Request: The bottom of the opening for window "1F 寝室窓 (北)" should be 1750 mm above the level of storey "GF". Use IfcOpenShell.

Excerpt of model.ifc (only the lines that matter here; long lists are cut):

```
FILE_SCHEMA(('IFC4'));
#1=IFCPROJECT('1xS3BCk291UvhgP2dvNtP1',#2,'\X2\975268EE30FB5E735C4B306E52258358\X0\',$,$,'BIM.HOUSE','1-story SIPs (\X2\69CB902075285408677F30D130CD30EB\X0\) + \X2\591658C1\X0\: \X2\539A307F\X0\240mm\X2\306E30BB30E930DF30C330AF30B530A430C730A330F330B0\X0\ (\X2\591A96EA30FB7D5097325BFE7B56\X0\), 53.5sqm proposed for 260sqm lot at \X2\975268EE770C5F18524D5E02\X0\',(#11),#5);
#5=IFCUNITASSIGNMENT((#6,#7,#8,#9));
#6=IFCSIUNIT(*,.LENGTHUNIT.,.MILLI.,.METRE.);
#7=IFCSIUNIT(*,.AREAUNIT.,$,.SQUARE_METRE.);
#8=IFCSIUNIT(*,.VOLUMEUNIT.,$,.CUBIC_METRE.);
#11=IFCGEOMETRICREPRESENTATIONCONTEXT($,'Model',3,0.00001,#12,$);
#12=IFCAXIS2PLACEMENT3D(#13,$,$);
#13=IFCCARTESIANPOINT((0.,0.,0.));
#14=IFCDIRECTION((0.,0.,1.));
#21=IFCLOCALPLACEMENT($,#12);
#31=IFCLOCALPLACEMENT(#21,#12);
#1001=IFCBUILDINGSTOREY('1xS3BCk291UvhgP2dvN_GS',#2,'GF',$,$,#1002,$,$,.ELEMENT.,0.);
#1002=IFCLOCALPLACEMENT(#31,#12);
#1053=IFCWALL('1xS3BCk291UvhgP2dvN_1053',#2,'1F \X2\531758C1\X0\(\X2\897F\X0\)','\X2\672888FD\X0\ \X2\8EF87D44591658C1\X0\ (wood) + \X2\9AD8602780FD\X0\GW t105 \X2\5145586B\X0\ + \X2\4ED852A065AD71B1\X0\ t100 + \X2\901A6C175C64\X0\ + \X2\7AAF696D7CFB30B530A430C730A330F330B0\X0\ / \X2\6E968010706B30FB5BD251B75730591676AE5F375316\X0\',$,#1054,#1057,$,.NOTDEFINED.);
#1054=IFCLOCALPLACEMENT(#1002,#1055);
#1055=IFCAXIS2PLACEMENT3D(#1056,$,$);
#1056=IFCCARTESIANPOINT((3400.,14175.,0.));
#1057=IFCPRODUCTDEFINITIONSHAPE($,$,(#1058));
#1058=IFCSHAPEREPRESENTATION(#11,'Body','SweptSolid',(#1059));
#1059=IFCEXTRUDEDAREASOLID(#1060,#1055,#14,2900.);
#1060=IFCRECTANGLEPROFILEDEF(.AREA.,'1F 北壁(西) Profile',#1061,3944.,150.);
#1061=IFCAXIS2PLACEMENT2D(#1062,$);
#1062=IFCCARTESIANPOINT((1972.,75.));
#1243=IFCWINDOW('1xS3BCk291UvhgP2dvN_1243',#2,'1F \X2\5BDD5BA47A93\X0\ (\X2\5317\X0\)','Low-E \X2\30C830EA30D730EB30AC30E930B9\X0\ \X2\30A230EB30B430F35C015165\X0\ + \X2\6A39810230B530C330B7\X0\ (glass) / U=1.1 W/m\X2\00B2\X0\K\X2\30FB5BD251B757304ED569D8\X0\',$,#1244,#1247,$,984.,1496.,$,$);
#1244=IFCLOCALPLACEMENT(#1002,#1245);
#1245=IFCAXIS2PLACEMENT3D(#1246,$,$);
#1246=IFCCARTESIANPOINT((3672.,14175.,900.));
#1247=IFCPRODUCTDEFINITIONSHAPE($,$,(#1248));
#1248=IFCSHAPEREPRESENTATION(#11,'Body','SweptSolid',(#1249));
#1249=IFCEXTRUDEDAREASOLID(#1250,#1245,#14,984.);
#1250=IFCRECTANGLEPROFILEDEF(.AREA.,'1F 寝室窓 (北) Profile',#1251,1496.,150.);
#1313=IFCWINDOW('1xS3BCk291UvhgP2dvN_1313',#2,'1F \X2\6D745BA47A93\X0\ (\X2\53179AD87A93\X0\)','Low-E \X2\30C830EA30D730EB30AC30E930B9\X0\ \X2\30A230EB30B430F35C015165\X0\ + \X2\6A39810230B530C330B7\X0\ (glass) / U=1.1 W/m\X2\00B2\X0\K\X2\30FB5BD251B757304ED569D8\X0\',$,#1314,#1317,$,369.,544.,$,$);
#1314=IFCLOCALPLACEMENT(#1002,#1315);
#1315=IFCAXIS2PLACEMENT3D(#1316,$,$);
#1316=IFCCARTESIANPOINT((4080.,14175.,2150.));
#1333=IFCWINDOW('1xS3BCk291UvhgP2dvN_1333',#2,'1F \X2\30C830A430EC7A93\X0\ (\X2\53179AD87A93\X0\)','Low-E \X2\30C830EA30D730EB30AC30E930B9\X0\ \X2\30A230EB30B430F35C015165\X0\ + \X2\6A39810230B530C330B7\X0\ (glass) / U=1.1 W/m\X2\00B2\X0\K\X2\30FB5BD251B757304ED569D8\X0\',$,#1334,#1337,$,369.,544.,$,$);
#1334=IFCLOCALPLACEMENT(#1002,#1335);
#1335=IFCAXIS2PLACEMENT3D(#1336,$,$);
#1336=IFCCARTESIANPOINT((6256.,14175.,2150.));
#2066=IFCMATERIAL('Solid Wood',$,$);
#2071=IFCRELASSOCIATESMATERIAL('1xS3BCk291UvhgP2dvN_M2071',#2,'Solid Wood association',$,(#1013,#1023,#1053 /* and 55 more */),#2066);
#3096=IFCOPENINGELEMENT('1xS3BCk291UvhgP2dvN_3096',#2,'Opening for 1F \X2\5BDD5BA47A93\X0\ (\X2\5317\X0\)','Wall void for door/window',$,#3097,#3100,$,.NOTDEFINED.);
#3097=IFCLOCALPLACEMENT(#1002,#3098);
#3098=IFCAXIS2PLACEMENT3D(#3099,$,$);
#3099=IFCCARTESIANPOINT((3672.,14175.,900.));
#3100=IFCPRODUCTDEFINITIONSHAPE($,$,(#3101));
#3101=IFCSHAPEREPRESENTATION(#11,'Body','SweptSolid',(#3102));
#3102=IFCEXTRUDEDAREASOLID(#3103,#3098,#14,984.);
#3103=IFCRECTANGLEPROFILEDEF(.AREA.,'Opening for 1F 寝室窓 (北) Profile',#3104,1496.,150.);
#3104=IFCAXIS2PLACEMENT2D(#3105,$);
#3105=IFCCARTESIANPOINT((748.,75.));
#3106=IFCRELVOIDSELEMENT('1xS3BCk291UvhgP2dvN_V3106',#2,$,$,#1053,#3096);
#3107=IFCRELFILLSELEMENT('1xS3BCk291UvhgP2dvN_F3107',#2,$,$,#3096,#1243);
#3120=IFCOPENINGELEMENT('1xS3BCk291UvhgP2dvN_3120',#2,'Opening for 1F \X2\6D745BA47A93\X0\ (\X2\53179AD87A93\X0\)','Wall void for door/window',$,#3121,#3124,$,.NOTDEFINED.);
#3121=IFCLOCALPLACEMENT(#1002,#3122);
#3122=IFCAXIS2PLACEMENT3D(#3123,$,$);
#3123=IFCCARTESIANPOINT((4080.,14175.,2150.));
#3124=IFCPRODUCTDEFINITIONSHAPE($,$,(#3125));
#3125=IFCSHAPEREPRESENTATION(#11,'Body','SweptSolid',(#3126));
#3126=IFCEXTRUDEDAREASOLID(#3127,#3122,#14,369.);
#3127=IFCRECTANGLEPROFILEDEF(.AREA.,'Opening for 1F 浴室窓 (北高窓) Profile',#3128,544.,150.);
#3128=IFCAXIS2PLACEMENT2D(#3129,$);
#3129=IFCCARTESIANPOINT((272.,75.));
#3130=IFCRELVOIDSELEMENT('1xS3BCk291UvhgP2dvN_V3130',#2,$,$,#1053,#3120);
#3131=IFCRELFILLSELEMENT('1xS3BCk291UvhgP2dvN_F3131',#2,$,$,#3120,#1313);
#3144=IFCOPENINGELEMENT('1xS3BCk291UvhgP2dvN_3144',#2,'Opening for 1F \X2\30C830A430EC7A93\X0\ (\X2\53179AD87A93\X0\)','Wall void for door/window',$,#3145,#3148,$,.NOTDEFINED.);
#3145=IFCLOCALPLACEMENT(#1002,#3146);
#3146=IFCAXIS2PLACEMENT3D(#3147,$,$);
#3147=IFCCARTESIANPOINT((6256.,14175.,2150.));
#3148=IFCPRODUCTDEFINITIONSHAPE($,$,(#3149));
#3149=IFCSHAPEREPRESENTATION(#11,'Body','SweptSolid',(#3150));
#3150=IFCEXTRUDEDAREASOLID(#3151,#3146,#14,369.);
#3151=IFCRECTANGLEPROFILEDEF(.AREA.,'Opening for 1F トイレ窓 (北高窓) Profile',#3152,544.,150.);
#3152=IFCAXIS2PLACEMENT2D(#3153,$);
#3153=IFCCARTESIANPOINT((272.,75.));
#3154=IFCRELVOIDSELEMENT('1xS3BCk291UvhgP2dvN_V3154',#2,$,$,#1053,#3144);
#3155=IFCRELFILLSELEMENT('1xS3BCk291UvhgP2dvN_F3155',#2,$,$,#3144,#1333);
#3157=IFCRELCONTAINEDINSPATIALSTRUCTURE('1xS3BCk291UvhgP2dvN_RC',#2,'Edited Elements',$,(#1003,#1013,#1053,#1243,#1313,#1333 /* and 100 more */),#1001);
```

```python
import numpy as np
import ifcopenshell
import ifcopenshell.api.geometry
import ifcopenshell.geom
import ifcopenshell.util.element
import ifcopenshell.util.placement
import ifcopenshell.util.shape
import ifcopenshell.util.unit

model = ifcopenshell.open("model.ifc")
unit_scale = ifcopenshell.util.unit.calculate_unit_scale(model)

window = model.by_guid("1xS3BCk291UvhgP2dvN_1243")
opening = window.FillsVoids[0].RelatingOpeningElement
storey = ifcopenshell.util.element.get_container(window, ifc_class="IfcBuildingStorey")
level = ifcopenshell.util.placement.get_local_placement(storey.ObjectPlacement)[2, 3]

# The opening's origin need not be at the sill, so measure its lowest point.
shape = ifcopenshell.geom.create_shape(ifcopenshell.geom.settings(), opening)
bottom = ifcopenshell.util.shape.get_shape_bottom_elevation(shape, shape.geometry) / unit_scale
dz = level + 1.75 / unit_scale - bottom

shift = np.array([0.0, 0.0, dz])
# The window is not placed relative to its opening, so move both.
for product in (opening, window):
    matrix = ifcopenshell.util.placement.get_local_placement(product.ObjectPlacement)
    matrix[:3, 3] += shift
    ifcopenshell.api.geometry.edit_object_placement(model, product=product, matrix=matrix, is_si=False)

print(f"moved by {dz * unit_scale:+.3f} m")

model.write("model_edited.ifc")
```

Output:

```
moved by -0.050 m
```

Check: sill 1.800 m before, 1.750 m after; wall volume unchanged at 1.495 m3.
